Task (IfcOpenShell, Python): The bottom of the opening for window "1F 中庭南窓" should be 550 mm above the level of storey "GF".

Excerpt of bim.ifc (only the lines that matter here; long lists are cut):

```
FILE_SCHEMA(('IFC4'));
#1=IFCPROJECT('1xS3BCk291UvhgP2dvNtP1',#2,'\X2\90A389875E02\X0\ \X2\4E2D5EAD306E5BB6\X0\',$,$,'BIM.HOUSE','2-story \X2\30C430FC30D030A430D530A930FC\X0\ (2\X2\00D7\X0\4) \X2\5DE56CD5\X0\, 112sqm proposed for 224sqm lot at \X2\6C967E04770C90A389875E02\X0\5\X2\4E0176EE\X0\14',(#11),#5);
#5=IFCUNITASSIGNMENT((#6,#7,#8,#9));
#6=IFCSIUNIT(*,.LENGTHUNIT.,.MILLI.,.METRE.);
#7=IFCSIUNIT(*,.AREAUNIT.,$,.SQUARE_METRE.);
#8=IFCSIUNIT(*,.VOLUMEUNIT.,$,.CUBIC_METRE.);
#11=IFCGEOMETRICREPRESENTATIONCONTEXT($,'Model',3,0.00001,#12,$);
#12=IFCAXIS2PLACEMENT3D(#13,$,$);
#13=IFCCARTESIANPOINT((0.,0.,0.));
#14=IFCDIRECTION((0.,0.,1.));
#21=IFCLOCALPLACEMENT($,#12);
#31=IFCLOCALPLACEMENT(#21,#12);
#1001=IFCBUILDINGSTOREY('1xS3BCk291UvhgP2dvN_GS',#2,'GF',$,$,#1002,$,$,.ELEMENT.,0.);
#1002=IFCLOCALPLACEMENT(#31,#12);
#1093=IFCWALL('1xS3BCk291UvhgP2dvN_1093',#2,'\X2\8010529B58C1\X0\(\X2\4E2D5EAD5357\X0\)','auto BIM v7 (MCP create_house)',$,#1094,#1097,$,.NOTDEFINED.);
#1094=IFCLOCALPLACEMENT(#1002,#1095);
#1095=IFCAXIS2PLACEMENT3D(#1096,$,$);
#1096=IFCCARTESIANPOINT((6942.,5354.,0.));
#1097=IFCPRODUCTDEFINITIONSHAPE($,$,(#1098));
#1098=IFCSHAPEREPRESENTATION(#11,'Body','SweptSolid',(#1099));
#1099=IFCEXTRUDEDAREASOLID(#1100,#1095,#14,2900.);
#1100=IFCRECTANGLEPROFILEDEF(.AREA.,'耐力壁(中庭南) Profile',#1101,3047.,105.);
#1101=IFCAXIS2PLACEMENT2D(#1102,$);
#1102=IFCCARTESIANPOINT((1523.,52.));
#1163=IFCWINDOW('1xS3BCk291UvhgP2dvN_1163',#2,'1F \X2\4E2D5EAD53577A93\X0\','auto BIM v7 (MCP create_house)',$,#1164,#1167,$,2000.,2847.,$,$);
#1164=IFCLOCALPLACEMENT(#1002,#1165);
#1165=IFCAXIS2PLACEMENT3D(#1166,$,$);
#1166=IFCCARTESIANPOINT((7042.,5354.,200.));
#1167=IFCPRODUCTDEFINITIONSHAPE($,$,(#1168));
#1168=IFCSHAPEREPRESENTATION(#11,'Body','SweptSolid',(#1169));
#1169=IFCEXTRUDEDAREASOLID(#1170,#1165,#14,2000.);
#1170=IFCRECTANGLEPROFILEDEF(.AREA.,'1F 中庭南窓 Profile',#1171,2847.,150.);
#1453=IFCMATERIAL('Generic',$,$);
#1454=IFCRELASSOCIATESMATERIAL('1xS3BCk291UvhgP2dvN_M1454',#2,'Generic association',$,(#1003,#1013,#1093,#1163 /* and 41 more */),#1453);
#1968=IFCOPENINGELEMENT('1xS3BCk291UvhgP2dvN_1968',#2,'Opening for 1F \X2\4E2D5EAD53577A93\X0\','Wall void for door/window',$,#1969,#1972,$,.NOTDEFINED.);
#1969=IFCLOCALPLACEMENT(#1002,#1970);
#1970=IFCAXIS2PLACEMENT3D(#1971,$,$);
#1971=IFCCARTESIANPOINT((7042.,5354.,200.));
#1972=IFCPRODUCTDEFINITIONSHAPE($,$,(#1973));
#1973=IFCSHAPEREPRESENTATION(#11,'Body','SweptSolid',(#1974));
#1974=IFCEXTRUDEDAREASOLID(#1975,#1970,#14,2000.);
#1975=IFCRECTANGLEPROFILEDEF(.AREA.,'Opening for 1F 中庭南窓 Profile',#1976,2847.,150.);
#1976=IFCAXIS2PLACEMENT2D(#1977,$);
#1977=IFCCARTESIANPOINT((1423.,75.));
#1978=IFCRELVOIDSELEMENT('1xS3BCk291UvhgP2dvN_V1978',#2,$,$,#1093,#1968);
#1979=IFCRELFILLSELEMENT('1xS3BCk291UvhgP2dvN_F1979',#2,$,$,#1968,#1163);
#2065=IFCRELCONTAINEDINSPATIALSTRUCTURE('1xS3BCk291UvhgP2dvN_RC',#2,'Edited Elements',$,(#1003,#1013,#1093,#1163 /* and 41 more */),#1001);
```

```python
import numpy as np
import ifcopenshell
import ifcopenshell.api.geometry
import ifcopenshell.geom
import ifcopenshell.util.element
import ifcopenshell.util.placement
import ifcopenshell.util.shape
import ifcopenshell.util.unit

model = ifcopenshell.open("bim.ifc")
unit_scale = ifcopenshell.util.unit.calculate_unit_scale(model)

window = model.by_guid("1xS3BCk291UvhgP2dvN_1163")
opening = window.FillsVoids[0].RelatingOpeningElement
storey = ifcopenshell.util.element.get_container(window, ifc_class="IfcBuildingStorey")
level = ifcopenshell.util.placement.get_local_placement(storey.ObjectPlacement)[2, 3]

# The opening's origin need not be at the sill, so measure its lowest point.
shape = ifcopenshell.geom.create_shape(ifcopenshell.geom.settings(), opening)
bottom = ifcopenshell.util.shape.get_shape_bottom_elevation(shape, shape.geometry) / unit_scale
dz = level + 550.0 - bottom

shift = np.array([0.0, 0.0, dz])
# The window is not placed relative to its opening, so move both.
for product in (opening, window):
    matrix = ifcopenshell.util.placement.get_local_placement(product.ObjectPlacement)
    matrix[:3, 3] += shift
    ifcopenshell.api.geometry.edit_object_placement(model, product=product, matrix=matrix, is_si=False)

print(f"moved by {dz * unit_scale:+.3f} m")

model.write("bim_v2.ifc")
```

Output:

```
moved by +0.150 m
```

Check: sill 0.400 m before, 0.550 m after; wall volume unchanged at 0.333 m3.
